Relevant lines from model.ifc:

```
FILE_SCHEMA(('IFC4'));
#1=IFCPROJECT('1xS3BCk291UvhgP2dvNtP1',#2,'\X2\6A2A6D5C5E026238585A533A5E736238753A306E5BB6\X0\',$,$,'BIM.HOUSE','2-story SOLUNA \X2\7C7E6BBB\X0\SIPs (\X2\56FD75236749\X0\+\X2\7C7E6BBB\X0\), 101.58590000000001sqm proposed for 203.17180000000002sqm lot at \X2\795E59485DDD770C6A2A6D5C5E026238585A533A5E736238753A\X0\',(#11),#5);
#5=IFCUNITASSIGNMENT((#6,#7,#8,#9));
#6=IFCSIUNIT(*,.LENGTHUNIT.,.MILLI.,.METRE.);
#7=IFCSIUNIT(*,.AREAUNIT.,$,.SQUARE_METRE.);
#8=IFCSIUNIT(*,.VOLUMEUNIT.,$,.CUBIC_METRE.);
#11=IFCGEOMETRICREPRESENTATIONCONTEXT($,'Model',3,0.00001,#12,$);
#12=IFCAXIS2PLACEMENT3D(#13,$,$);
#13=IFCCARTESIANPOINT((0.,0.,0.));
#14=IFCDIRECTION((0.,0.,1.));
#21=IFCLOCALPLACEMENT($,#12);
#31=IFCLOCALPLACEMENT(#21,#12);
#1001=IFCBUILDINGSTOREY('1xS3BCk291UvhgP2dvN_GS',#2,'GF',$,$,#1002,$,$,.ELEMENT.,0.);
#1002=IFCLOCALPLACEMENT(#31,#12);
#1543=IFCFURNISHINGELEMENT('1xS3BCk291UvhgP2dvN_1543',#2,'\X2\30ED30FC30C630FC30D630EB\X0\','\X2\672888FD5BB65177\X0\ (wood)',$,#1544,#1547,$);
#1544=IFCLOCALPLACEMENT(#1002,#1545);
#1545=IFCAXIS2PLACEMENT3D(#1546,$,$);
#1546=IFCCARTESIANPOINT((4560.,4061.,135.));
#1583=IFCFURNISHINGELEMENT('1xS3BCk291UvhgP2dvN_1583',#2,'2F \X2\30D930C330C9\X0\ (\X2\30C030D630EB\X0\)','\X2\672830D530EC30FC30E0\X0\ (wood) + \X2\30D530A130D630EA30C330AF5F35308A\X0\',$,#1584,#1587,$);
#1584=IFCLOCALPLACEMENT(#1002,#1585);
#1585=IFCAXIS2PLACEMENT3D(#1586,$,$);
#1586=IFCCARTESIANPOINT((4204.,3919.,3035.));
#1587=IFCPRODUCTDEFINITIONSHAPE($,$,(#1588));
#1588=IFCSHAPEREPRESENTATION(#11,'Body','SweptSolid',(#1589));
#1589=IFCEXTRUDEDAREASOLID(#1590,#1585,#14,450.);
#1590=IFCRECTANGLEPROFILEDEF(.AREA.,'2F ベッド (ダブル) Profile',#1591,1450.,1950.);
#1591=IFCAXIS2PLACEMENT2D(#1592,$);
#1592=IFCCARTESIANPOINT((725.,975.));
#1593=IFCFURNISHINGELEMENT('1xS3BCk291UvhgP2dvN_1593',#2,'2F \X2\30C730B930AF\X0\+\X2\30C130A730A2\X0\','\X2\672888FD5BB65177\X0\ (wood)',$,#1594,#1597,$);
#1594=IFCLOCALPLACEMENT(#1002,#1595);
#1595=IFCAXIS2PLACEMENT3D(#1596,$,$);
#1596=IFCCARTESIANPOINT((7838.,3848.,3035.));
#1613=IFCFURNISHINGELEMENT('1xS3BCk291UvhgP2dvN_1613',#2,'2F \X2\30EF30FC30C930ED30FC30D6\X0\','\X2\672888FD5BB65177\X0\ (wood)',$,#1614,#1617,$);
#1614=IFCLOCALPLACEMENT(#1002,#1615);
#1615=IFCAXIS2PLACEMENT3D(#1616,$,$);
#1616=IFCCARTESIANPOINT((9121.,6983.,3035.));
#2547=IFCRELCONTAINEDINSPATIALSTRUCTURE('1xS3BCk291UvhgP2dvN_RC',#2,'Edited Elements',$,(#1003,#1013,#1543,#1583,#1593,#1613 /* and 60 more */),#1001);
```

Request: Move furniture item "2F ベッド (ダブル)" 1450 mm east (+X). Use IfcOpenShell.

```python
import ifcopenshell
import ifcopenshell.api.geometry
import ifcopenshell.util.placement
import ifcopenshell.util.unit

model = ifcopenshell.open("model.ifc")
unit_scale = ifcopenshell.util.unit.calculate_unit_scale(model)

item = model.by_guid("1xS3BCk291UvhgP2dvN_1583")
matrix = ifcopenshell.util.placement.get_local_placement(item.ObjectPlacement)
matrix[0, 3] += 1.45 / unit_scale
ifcopenshell.api.geometry.edit_object_placement(model, product=item, matrix=matrix, is_si=False)

print(ifcopenshell.util.placement.get_local_placement(item.ObjectPlacement).round(3) + 0.0)

model.write("model_v2.ifc")
```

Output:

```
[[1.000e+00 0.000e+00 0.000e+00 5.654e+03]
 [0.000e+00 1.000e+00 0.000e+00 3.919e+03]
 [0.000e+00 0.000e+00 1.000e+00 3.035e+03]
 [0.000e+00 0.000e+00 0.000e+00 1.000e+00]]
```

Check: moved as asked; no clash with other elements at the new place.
